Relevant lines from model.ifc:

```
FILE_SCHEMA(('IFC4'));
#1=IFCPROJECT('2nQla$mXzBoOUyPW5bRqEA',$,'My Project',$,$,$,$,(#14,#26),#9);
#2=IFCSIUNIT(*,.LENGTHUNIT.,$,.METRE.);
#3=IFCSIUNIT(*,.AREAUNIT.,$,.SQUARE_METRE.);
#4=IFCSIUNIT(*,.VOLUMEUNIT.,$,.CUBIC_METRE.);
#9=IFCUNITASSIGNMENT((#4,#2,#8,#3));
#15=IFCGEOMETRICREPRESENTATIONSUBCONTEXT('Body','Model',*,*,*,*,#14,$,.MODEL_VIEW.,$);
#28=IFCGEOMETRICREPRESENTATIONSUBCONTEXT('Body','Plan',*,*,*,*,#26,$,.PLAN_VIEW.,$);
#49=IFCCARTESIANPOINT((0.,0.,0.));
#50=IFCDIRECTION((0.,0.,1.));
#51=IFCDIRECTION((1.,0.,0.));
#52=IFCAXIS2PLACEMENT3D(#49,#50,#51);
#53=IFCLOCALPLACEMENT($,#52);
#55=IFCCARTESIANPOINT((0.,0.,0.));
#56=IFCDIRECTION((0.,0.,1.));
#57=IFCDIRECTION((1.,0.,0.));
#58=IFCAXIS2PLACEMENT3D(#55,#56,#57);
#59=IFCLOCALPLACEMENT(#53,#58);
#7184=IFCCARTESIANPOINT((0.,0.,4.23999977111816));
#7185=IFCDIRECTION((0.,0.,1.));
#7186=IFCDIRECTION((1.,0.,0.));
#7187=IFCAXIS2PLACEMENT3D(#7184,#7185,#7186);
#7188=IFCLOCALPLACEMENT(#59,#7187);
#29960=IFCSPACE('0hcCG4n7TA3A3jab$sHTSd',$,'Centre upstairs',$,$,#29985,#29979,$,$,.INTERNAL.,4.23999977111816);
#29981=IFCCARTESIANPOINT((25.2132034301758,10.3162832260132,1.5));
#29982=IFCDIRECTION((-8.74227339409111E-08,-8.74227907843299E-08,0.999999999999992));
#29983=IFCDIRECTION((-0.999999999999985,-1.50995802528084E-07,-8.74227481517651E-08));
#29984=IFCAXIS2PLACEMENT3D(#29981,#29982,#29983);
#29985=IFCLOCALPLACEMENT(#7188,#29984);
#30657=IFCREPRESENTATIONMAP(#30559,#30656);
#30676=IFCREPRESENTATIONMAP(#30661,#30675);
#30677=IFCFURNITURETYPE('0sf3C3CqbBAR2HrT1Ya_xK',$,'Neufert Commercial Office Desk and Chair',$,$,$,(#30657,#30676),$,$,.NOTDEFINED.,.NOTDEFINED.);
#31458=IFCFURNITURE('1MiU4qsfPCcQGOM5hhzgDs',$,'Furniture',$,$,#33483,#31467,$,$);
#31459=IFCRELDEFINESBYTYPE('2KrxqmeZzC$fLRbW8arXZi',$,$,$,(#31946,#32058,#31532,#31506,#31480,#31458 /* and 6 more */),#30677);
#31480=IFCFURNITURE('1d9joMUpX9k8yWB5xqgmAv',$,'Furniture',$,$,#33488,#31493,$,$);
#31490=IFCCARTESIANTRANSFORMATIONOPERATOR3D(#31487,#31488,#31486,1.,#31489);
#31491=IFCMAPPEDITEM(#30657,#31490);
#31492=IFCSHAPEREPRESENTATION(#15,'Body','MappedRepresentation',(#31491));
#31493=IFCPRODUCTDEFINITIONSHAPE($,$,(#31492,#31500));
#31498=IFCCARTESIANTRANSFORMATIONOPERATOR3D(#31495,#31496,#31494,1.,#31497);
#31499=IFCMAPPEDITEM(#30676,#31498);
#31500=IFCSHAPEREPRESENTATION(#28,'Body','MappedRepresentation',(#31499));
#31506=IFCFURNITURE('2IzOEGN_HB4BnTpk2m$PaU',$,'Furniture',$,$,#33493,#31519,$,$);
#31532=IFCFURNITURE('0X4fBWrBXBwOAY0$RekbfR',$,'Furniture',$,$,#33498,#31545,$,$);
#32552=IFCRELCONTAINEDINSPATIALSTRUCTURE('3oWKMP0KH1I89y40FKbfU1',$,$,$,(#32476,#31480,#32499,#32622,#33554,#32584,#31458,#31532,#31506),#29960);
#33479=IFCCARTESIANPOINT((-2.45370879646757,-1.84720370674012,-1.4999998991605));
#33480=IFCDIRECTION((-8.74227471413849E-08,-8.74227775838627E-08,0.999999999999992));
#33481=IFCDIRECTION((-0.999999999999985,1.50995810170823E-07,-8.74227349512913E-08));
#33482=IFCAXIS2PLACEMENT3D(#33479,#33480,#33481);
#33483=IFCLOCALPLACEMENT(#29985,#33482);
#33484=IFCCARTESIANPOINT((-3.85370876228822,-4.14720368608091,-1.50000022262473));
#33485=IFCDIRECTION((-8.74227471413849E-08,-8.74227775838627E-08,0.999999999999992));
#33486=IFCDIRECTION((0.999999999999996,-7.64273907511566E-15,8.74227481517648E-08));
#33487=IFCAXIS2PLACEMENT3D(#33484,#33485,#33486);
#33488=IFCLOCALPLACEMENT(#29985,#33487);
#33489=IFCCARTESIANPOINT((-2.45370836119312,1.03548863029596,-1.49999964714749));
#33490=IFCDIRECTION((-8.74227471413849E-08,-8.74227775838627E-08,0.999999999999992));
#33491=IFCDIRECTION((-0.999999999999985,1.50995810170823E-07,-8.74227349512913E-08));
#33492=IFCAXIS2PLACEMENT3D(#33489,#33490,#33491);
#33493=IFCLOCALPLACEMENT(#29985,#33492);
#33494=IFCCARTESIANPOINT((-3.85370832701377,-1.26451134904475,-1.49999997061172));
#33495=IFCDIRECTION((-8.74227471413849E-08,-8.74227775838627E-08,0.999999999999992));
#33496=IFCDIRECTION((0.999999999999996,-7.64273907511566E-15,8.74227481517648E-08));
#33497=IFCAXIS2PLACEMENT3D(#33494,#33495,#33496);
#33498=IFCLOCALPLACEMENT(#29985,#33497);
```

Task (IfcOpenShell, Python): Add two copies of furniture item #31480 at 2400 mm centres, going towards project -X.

```python
import numpy as np
import ifcopenshell
import ifcopenshell.api.geometry
import ifcopenshell.api.root
import ifcopenshell.util.element
import ifcopenshell.util.placement
import ifcopenshell.util.unit

model = ifcopenshell.open("model.ifc")
unit_scale = ifcopenshell.util.unit.calculate_unit_scale(model)

source = model.by_guid("1d9joMUpX9k8yWB5xqgmAv")
base = ifcopenshell.util.placement.get_local_placement(source.ObjectPlacement)
step = np.array([-1.0, 0.0, 0.0]) * 2.4 / unit_scale

for i in range(1, 3):
    copy = ifcopenshell.api.root.copy_class(model, product=source)
    copy.Representation = ifcopenshell.util.element.copy_deep(
        model, source.Representation, exclude=["IfcGeometricRepresentationContext", "IfcRepresentationMap"]
    )
    matrix = base.copy()
    matrix[:3, 3] += i * step
    print("added at", matrix[:3, 3].round(3) + 0.0)
    ifcopenshell.api.geometry.edit_object_placement(model, product=copy, matrix=matrix, is_si=False)

model.write("model_rev.ifc")
```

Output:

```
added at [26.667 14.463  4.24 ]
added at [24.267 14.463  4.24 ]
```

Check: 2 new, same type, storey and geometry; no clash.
